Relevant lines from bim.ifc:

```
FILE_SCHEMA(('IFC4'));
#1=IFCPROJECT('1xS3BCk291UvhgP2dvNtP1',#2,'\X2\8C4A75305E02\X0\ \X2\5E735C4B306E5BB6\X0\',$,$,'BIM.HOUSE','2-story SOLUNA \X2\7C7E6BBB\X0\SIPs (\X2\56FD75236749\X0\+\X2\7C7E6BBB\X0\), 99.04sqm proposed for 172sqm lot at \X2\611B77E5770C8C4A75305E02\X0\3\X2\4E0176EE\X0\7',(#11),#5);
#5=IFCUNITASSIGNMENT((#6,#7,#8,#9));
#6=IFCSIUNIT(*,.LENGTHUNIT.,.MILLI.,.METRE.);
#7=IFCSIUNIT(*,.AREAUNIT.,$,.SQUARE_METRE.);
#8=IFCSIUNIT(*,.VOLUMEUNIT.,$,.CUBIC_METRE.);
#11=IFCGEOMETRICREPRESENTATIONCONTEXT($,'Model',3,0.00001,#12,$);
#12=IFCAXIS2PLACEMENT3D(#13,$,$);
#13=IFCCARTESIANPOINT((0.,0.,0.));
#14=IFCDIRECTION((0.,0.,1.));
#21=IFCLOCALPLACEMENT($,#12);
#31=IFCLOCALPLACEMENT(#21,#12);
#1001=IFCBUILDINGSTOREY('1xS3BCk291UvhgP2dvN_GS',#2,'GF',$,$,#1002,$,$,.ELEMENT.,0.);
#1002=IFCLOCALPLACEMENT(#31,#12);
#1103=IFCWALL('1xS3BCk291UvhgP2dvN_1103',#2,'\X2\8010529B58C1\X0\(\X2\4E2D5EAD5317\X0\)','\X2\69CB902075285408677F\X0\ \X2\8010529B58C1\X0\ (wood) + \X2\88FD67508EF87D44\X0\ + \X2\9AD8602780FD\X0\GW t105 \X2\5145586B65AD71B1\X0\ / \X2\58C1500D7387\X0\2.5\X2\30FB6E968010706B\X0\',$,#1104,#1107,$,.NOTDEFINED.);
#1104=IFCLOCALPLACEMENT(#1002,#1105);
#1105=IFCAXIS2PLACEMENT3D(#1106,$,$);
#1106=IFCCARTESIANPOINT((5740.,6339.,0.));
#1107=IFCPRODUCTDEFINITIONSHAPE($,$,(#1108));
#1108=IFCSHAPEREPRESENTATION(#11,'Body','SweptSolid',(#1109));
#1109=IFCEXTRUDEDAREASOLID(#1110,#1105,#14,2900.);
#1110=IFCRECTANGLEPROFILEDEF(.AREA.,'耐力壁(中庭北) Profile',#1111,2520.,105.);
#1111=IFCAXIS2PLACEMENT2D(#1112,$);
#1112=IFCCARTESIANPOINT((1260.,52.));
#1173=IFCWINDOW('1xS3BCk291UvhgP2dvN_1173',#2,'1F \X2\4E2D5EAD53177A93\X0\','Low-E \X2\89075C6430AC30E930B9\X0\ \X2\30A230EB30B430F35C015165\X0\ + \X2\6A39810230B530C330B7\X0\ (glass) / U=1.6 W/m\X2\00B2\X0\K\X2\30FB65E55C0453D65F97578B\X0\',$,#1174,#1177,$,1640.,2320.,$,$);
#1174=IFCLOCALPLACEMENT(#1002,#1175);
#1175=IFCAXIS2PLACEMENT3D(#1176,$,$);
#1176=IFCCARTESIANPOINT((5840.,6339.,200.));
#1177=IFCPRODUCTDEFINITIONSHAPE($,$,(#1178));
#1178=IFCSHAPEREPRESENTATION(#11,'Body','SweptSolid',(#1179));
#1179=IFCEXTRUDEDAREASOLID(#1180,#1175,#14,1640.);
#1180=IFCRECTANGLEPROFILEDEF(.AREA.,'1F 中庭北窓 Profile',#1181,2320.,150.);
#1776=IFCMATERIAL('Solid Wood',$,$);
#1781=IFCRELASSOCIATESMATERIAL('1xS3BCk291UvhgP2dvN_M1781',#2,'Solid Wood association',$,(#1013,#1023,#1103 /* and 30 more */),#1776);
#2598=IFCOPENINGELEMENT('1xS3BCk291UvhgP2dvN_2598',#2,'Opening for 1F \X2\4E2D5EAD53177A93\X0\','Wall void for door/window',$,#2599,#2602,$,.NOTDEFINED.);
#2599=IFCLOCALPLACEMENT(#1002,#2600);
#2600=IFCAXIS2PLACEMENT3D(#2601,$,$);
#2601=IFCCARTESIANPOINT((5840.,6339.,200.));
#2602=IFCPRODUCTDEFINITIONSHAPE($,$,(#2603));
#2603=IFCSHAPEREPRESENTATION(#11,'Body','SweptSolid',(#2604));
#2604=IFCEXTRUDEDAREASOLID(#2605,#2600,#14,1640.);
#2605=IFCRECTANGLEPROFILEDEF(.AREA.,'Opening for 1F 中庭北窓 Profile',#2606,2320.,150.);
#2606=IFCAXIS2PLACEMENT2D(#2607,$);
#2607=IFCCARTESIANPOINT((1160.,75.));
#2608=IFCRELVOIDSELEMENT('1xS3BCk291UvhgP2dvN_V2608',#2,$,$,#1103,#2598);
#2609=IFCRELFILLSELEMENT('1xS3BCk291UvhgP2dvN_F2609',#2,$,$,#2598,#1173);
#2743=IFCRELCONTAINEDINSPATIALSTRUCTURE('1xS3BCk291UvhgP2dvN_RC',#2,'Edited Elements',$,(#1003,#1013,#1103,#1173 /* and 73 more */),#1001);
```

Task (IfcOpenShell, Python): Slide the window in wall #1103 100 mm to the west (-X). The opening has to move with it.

```python
import ifcopenshell
import ifcopenshell.api.geometry
import ifcopenshell.util.placement
import ifcopenshell.util.unit

model = ifcopenshell.open("bim.ifc")
unit_scale = ifcopenshell.util.unit.calculate_unit_scale(model)

window = model.by_guid("1xS3BCk291UvhgP2dvN_1173")
opening = window.FillsVoids[0].RelatingOpeningElement
wall = opening.VoidsElements[0].RelatingBuildingElement

wall_matrix = ifcopenshell.util.placement.get_local_placement(wall.ObjectPlacement)
shift = wall_matrix[:3, 0] * -0.1 / unit_scale
before = ifcopenshell.util.placement.get_local_placement(window.ObjectPlacement)[:3, 3].copy()

# The window is not placed relative to its opening, so move both.
for product in (opening, window):
    matrix = ifcopenshell.util.placement.get_local_placement(product.ObjectPlacement)
    matrix[:3, 3] += shift
    ifcopenshell.api.geometry.edit_object_placement(model, product=product, matrix=matrix, is_si=False)

after = ifcopenshell.util.placement.get_local_placement(window.ObjectPlacement)[:3, 3]
print("window moved by", (after - before).round(3) + 0.0)

model.write("bim_updated.ifc")
```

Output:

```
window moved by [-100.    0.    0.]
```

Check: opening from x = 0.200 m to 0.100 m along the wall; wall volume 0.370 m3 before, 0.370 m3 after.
